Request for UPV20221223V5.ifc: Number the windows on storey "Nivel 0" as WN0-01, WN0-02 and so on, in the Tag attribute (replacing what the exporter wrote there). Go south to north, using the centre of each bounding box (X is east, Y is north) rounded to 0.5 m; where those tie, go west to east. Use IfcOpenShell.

First a look at what the model holds.

```python
import ifcopenshell
import ifcopenshell.util.element
import ifcopenshell.util.placement

model = ifcopenshell.open("UPV20221223V5.ifc")
print(model.schema)
storey = next(s for s in model.by_type("IfcBuildingStorey") if s.Name == "Nivel 0")
windows = [e for e in ifcopenshell.util.element.get_decomposition(storey) if e.is_a("IfcWindow")]
for e in sorted(windows, key=lambda e: e.id()):
    origin = ifcopenshell.util.placement.get_local_placement(e.ObjectPlacement)[:3, 3]
    print(e.id(), e.Tag, e.Name, origin.round(2) + 0.0, sep=" | ")
```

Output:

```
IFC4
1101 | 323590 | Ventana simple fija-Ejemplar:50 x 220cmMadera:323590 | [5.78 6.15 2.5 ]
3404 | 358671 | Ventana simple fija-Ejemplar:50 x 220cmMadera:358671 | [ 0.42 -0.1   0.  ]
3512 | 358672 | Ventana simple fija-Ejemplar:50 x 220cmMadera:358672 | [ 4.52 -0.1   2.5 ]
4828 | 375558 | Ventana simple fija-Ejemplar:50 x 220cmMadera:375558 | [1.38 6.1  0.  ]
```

```python
import ifcopenshell
import ifcopenshell.geom
import ifcopenshell.util.element
import ifcopenshell.util.shape

model = ifcopenshell.open("UPV20221223V5.ifc")
settings = ifcopenshell.geom.settings()
settings.set("use-world-coords", True)


def centre(element):
    shape = ifcopenshell.geom.create_shape(settings, element)
    return ifcopenshell.util.shape.get_bbox_centroid(shape.geometry)


storey = next(s for s in model.by_type("IfcBuildingStorey") if s.Name == "Nivel 0")
windows = [e for e in ifcopenshell.util.element.get_decomposition(storey) if e.is_a("IfcWindow")]

# Insertion points can sit at a corner or the storey origin, so sort by the geometry (in metres).
centres = {e: centre(e) for e in windows}
windows.sort(key=lambda e: (round(centres[e][1] / 0.5), centres[e][0]))

for i, e in enumerate(windows, start=1):
    number = f"WN0-{i:02d}"
    e.Tag = number
    print(e.id(), number)

model.write("UPV20221223V5_edited.ifc")
```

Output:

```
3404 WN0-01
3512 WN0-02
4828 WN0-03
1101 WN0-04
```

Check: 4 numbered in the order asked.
